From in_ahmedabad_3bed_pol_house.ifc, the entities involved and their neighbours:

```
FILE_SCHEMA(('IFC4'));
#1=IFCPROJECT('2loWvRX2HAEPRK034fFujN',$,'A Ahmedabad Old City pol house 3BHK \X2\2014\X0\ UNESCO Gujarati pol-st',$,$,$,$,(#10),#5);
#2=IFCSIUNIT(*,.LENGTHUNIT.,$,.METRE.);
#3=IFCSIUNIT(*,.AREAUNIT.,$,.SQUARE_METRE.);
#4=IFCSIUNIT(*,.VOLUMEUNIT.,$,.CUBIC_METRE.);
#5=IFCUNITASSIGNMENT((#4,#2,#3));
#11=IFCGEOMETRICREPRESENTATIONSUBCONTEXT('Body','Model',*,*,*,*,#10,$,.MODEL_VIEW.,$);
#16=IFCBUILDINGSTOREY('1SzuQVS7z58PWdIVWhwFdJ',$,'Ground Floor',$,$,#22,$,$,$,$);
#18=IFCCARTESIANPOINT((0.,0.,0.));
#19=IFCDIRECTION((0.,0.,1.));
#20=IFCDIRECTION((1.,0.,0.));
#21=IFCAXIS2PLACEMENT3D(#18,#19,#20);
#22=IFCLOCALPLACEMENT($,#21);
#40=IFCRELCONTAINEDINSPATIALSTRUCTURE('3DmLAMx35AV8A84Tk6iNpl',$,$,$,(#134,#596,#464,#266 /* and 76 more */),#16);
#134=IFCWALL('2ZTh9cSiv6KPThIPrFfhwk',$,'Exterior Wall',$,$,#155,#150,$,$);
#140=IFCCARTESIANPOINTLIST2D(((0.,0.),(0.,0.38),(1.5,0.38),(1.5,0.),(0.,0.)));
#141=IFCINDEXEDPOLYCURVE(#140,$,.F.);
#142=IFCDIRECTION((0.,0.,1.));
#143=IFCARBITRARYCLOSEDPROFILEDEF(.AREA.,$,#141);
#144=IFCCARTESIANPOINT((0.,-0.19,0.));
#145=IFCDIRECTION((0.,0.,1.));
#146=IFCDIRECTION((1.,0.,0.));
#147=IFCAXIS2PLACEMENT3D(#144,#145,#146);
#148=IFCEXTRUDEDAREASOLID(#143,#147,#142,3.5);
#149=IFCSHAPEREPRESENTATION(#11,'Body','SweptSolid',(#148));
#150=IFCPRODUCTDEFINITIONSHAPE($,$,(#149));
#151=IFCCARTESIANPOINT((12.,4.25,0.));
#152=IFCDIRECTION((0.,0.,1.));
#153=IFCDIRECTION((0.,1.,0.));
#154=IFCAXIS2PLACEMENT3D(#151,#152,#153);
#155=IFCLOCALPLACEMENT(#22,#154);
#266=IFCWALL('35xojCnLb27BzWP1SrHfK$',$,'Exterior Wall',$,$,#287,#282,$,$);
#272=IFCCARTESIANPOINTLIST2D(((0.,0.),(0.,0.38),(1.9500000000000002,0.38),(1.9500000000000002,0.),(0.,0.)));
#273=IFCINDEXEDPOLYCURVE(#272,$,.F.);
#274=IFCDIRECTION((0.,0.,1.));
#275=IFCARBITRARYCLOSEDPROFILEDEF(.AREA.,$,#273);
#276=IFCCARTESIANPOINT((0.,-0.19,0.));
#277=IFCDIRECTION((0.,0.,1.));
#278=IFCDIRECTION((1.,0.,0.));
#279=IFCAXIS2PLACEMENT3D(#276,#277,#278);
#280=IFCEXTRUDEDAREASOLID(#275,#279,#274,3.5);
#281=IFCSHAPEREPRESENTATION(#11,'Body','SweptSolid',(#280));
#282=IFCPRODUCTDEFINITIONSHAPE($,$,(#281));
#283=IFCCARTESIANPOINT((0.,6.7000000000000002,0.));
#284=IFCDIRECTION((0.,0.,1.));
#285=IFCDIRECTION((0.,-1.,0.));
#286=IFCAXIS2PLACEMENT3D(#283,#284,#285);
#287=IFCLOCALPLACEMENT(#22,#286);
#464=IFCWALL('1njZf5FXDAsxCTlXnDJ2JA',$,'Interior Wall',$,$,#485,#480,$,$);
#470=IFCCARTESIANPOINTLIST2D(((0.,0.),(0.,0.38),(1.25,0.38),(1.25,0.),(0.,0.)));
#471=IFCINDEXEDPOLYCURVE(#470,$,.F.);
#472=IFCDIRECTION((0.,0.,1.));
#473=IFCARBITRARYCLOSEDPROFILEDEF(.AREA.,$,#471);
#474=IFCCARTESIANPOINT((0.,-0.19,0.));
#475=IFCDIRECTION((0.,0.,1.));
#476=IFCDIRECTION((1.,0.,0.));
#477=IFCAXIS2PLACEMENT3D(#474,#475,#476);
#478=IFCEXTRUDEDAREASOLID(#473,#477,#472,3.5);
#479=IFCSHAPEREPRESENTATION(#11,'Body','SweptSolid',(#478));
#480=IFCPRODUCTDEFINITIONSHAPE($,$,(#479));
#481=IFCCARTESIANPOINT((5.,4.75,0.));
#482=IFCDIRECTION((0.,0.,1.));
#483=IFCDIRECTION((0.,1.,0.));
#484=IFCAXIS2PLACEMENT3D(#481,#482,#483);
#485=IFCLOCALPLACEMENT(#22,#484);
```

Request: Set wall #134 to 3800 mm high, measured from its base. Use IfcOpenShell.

```python
import ifcopenshell
import ifcopenshell.geom
import ifcopenshell.util.representation
import ifcopenshell.util.shape
import ifcopenshell.util.unit

model = ifcopenshell.open("in_ahmedabad_3bed_pol_house.ifc")
unit_scale = ifcopenshell.util.unit.calculate_unit_scale(model)
settings = ifcopenshell.geom.settings()


def volume(element):
    """Net volume in cubic metres, openings subtracted."""
    shape = ifcopenshell.geom.create_shape(settings, element)
    return ifcopenshell.util.shape.get_volume(shape.geometry)


wall = model.by_id(134)
before = volume(wall)

body = ifcopenshell.util.representation.get_representation(wall, "Model", "Body")
solid = body.Items[0]
old_height = solid.Depth
solid.Depth = 3.8 / unit_scale
after = volume(wall)

print(f"height {old_height:g} -> {solid.Depth:g}, volume {before:.3f} -> {after:.3f} m3")

model.write("in_ahmedabad_3bed_pol_house_edited.ifc")
```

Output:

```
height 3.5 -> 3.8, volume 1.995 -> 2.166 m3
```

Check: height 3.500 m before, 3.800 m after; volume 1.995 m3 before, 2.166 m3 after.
